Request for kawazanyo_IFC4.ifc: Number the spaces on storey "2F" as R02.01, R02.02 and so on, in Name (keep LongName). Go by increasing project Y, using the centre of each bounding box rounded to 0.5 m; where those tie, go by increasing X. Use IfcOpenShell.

First a look at what the model holds.

```python
import ifcopenshell
import ifcopenshell.util.element
import ifcopenshell.util.placement

model = ifcopenshell.open("kawazanyo_IFC4.ifc")
print(model.schema)
storey = next(s for s in model.by_type("IfcBuildingStorey") if s.Name == "2F")
spaces = [e for e in ifcopenshell.util.element.get_decomposition(storey) if e.is_a("IfcSpace")]
for e in sorted(spaces, key=lambda e: e.id()):
    origin = ifcopenshell.util.placement.get_local_placement(e.ObjectPlacement)[:3, 3]
    print(e.id(), e.Name, e.LongName, origin.round(2) + 0.0, sep=" | ")
```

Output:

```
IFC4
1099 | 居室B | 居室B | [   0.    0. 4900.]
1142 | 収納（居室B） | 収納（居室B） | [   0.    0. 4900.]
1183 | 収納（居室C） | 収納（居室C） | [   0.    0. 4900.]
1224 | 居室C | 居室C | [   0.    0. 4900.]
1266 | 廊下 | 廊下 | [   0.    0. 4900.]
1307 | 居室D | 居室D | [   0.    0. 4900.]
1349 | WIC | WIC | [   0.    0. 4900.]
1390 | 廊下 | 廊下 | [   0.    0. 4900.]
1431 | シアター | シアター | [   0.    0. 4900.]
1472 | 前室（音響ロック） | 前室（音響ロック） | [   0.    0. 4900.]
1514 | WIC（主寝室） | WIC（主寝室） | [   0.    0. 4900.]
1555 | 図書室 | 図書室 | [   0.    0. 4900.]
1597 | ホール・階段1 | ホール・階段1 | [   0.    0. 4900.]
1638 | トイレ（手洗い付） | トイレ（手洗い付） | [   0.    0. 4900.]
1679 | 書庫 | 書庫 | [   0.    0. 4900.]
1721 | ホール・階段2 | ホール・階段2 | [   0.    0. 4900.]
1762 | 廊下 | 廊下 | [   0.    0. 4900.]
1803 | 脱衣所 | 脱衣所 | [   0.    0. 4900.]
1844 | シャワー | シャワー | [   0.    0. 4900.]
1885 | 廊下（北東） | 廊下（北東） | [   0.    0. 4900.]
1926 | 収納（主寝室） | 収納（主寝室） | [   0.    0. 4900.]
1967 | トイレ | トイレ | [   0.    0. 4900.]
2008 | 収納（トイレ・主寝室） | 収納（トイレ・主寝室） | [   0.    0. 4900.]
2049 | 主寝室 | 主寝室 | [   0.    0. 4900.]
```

```python
import ifcopenshell
import ifcopenshell.geom
import ifcopenshell.util.element
import ifcopenshell.util.shape

model = ifcopenshell.open("kawazanyo_IFC4.ifc")
settings = ifcopenshell.geom.settings()
settings.set("use-world-coords", True)


def centre(element):
    shape = ifcopenshell.geom.create_shape(settings, element)
    return ifcopenshell.util.shape.get_bbox_centroid(shape.geometry)


storey = next(s for s in model.by_type("IfcBuildingStorey") if s.Name == "2F")
spaces = [e for e in ifcopenshell.util.element.get_decomposition(storey) if e.is_a("IfcSpace")]

# Insertion points can sit at a corner or the storey origin, so sort by the geometry (in metres).
centres = {e: centre(e) for e in spaces}
spaces.sort(key=lambda e: (round(centres[e][1] / 0.5), centres[e][0]))

for i, e in enumerate(spaces, start=1):
    number = f"R02.{i:02d}"
    e.Name = number
    print(e.id(), number)

model.write("kawazanyo_IFC4_edited.ifc")
```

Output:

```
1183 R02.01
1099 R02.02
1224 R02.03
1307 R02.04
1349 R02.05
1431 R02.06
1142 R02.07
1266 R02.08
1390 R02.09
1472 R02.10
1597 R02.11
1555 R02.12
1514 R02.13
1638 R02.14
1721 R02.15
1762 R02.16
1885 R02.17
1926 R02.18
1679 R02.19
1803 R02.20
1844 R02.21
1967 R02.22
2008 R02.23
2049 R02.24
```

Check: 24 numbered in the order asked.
